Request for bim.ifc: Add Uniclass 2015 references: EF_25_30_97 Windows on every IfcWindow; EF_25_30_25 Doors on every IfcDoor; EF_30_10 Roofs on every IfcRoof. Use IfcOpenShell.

First a look at what the model holds.

```python
import ifcopenshell

model = ifcopenshell.open("bim.ifc")
print(model.schema)
print("classifications:", [c.Name for c in model.by_type("IfcClassification")])
for ifc_class in ("IfcDoor", "IfcRoof", "IfcStair", "IfcWall", "IfcWindow"):
    print(ifc_class, len(model.by_type(ifc_class)))
```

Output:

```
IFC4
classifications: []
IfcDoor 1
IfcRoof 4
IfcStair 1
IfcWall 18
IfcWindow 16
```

```python
import ifcopenshell
import ifcopenshell.api.classification

model = ifcopenshell.open("bim.ifc")

system = ifcopenshell.api.classification.add_classification(model, classification="Uniclass 2015")

codes = {
    "IfcWindow": ("EF_25_30_97", "Windows"),
    "IfcDoor": ("EF_25_30_25", "Doors"),
    "IfcRoof": ("EF_30_10", "Roofs"),
}
for ifc_class, (code, name) in codes.items():
    products = model.by_type(ifc_class)
    ifcopenshell.api.classification.add_reference(
        model, products=products, classification=system, identification=code, name=name
    )
    print(code, len(products))

model.write("bim-out.ifc")
```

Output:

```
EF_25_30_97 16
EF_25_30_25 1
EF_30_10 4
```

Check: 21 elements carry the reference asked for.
